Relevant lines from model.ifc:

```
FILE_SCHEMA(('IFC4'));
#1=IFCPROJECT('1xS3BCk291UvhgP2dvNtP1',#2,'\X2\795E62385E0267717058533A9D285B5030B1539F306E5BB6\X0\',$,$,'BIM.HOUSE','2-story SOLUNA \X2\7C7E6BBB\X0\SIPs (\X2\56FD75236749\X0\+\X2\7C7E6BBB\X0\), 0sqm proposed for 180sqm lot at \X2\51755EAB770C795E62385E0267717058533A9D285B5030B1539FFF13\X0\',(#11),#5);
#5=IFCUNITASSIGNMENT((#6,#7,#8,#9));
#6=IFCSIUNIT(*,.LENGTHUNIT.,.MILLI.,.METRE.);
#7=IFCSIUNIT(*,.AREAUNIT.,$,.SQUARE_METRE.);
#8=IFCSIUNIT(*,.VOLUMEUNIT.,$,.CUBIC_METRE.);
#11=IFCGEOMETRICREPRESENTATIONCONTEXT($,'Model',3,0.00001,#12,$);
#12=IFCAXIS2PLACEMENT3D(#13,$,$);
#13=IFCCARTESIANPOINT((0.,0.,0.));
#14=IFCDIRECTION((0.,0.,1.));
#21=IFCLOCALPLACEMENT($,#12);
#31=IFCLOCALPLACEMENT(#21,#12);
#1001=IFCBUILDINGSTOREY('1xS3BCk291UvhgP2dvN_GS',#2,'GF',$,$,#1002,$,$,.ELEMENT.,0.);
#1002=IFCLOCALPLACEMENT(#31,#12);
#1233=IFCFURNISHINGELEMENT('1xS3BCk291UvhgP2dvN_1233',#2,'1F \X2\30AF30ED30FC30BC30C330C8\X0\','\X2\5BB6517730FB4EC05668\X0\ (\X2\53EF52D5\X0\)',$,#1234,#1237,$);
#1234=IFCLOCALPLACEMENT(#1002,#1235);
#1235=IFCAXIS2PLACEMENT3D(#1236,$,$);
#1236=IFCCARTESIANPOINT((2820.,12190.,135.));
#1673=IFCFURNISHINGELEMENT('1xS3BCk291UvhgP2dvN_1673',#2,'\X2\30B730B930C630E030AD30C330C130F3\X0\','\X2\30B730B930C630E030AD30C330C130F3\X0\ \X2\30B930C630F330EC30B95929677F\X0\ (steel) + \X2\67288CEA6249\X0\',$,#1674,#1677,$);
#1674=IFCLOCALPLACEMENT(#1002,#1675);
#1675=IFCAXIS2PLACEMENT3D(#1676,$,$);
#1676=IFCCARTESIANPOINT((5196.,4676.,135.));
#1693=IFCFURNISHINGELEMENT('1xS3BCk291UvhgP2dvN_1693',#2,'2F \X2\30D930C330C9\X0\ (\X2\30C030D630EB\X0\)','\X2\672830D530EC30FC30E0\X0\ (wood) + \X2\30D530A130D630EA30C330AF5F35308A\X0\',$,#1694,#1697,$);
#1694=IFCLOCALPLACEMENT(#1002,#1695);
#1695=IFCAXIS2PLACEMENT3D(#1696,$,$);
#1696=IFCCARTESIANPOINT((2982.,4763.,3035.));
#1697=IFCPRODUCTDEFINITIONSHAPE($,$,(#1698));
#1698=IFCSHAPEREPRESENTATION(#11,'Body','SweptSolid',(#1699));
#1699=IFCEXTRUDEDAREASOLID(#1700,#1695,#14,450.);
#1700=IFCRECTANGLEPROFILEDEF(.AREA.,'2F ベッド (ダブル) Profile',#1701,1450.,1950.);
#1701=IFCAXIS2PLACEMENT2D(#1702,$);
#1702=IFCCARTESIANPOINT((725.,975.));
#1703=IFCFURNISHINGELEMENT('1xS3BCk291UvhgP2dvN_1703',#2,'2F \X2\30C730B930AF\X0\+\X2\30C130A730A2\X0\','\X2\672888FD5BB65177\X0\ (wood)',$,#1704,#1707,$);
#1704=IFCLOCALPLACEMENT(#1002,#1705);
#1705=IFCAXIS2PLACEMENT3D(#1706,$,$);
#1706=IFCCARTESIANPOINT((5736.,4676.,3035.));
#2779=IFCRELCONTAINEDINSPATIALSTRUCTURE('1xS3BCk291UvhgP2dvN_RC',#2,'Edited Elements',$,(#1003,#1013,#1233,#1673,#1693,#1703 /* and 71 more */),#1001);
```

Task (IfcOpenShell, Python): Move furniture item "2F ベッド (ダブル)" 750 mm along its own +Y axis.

```python
import ifcopenshell
import ifcopenshell.api.geometry
import ifcopenshell.util.placement
import ifcopenshell.util.unit

model = ifcopenshell.open("model.ifc")
unit_scale = ifcopenshell.util.unit.calculate_unit_scale(model)

item = model.by_id(1693)
matrix = ifcopenshell.util.placement.get_local_placement(item.ObjectPlacement)
matrix[:3, 3] += matrix[:3, 1] * 0.75 / unit_scale
ifcopenshell.api.geometry.edit_object_placement(model, product=item, matrix=matrix, is_si=False)

print(ifcopenshell.util.placement.get_local_placement(item.ObjectPlacement).round(3) + 0.0)

model.write("model_rev.ifc")
```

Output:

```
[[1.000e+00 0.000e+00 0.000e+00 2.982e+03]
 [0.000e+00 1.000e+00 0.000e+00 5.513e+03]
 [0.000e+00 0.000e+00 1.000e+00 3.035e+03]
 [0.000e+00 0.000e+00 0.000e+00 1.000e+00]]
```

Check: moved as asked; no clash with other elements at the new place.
